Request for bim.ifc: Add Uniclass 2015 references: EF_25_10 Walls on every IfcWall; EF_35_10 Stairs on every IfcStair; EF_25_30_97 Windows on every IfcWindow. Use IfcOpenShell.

First a look at what the model holds.

```python
import ifcopenshell

model = ifcopenshell.open("bim.ifc")
print(model.schema)
print("classifications:", [c.Name for c in model.by_type("IfcClassification")])
for ifc_class in ("IfcDoor", "IfcRoof", "IfcStair", "IfcWall", "IfcWindow"):
    print(ifc_class, len(model.by_type(ifc_class)))
```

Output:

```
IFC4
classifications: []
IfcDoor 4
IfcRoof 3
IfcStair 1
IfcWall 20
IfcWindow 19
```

```python
import ifcopenshell
import ifcopenshell.api.classification

model = ifcopenshell.open("bim.ifc")

system = ifcopenshell.api.classification.add_classification(model, classification="Uniclass 2015")

codes = {
    "IfcWall": ("EF_25_10", "Walls"),
    "IfcStair": ("EF_35_10", "Stairs"),
    "IfcWindow": ("EF_25_30_97", "Windows"),
}
for ifc_class, (code, name) in codes.items():
    products = model.by_type(ifc_class)
    ifcopenshell.api.classification.add_reference(
        model, products=products, classification=system, identification=code, name=name
    )
    print(code, len(products))

model.write("bim_edited.ifc")
```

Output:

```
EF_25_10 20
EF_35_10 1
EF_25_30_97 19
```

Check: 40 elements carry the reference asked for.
